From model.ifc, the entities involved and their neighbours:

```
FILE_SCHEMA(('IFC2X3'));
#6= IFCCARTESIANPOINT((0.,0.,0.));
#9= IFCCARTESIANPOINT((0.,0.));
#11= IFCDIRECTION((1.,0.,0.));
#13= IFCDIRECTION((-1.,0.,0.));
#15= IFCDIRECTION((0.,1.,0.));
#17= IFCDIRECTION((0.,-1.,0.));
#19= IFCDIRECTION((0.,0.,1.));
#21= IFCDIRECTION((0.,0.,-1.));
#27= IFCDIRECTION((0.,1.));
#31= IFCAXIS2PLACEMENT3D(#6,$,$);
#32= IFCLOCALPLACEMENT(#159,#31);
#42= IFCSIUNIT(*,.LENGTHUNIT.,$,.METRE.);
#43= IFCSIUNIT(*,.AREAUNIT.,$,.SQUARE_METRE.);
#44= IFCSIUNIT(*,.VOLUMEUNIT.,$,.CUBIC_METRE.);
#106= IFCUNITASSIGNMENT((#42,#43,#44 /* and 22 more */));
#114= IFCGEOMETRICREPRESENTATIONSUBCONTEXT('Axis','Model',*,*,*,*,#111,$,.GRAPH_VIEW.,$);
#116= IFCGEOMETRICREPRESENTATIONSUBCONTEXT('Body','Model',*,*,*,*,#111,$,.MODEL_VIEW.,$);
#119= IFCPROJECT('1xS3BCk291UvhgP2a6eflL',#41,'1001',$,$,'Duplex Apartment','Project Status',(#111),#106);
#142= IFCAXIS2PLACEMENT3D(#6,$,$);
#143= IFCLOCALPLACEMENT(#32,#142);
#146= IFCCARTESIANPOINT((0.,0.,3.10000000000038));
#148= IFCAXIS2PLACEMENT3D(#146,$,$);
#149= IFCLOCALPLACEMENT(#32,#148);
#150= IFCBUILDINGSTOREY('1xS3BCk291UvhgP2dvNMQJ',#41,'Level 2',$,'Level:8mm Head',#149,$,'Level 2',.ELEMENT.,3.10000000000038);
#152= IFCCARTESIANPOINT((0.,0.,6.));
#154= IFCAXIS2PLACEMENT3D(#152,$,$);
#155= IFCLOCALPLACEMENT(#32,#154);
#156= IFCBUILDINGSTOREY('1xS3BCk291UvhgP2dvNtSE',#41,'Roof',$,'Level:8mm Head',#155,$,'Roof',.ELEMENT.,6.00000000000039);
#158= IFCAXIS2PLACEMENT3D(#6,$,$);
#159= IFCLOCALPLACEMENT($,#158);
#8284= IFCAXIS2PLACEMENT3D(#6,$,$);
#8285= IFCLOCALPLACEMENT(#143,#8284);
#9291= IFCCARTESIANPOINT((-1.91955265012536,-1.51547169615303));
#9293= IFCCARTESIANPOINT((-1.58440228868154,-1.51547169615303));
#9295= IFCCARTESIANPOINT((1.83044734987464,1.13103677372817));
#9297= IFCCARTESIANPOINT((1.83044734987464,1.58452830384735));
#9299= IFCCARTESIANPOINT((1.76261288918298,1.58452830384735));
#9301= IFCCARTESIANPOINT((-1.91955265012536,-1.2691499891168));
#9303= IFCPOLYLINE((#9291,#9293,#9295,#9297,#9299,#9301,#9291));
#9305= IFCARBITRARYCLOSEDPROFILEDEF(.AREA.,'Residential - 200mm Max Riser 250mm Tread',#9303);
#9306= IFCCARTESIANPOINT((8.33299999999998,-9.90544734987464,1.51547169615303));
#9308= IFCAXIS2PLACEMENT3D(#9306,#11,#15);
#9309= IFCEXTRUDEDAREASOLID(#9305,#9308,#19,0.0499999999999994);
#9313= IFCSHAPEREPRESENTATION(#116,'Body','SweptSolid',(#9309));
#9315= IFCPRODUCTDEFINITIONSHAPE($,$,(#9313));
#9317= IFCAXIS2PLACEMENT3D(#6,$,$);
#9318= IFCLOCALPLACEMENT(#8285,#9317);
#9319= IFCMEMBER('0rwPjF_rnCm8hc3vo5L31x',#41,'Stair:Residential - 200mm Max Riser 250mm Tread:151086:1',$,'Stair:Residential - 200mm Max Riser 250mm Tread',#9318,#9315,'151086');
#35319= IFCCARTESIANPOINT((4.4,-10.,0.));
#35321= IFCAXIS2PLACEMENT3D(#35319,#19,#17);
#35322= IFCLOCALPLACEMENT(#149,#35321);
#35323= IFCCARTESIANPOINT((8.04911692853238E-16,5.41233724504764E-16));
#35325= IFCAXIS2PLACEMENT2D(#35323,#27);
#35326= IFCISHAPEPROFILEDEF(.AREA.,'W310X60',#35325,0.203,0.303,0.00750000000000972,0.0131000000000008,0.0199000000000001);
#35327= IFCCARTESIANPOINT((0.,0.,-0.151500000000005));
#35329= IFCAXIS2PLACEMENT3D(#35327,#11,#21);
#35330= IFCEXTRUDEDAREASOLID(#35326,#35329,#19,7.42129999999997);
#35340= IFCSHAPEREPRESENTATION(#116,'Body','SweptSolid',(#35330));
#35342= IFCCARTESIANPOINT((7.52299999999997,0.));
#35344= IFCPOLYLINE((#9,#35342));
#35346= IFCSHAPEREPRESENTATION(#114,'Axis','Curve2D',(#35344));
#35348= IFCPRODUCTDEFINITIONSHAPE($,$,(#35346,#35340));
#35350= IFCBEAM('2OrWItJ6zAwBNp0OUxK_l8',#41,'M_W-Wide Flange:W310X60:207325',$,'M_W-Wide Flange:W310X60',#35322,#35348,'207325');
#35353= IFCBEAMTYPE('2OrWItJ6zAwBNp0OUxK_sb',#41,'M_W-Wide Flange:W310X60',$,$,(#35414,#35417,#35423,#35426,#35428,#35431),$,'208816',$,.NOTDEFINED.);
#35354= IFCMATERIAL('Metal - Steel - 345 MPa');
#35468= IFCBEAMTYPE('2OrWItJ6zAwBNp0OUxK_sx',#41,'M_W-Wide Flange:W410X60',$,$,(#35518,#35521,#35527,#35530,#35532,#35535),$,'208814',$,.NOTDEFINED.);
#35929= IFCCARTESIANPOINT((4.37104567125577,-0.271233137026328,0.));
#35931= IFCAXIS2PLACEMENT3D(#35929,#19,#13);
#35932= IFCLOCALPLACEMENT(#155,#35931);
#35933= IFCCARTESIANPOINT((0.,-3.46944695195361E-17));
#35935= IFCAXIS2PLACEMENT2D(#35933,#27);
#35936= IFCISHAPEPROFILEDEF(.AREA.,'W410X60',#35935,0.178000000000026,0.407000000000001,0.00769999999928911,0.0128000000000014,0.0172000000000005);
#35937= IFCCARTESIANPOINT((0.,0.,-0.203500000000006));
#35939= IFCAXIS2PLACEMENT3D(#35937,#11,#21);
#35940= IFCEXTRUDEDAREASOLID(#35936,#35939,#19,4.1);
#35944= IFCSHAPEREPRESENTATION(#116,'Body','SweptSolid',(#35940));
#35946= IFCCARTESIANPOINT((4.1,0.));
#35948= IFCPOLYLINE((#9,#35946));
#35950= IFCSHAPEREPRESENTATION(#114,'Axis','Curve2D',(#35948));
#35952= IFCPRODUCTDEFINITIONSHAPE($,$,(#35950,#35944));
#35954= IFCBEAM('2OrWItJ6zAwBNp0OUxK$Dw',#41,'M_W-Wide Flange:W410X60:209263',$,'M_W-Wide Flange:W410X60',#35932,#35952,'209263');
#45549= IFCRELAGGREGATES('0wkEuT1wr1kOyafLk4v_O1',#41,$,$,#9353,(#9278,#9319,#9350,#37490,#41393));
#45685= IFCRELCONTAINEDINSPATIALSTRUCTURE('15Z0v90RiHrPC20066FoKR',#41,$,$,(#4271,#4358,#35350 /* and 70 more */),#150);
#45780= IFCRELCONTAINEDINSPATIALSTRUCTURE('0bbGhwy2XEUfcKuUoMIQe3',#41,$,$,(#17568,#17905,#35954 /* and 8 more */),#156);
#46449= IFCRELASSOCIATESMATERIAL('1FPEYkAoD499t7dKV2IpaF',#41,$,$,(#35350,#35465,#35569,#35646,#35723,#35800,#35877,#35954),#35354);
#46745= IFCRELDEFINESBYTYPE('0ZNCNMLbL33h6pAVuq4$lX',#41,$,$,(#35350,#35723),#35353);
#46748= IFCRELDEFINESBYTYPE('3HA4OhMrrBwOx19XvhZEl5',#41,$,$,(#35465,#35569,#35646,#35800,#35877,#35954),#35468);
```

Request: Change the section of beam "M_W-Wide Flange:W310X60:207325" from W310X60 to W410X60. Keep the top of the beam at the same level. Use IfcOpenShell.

```python
import ifcopenshell
import ifcopenshell.api.type
import ifcopenshell.util.element
import ifcopenshell.util.representation

model = ifcopenshell.open("model.ifc")

member = model.by_guid("2OrWItJ6zAwBNp0OUxK_l8")
source = next(p for p in model.by_type("IfcIShapeProfileDef") if p.ProfileName == "W410X60")

body = ifcopenshell.util.representation.get_representation(member, "Model", "Body")
solid = body.Items[0]
old_profile = solid.SweptArea

# Copy the section's sizes but keep this member's own profile position.
profile = ifcopenshell.util.element.copy(model, source)
# Profiles are centred, so shift by half the change in depth to hold the top.
shift = (old_profile.OverallDepth - profile.OverallDepth) / 2
x, y = old_profile.Position.Location.Coordinates
up = (-1.0, 0.0)  # upwards, in the solid's own plane
location = model.createIfcCartesianPoint((x + up[0] * shift, y + up[1] * shift))
profile.Position = model.createIfcAxis2Placement2D(location, old_profile.Position.RefDirection)
solid.SweptArea = profile
if not model.get_total_inverses(old_profile):
    ifcopenshell.util.element.remove_deep2(model, old_profile)

new_type = model.by_guid("2OrWItJ6zAwBNp0OUxK_sx")
ifcopenshell.api.type.assign_type(
    model, related_objects=[member], relating_type=new_type, should_map_representations=False
)
member.Name = member.Name.replace("W310X60", "W410X60")
member.ObjectType = "M_W-Wide Flange:W410X60"

print(solid.SweptArea)

model.write("model_v2.ifc")
```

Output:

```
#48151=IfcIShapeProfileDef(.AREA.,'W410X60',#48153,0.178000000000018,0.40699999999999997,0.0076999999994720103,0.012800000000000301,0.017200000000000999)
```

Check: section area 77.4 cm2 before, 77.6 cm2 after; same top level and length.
